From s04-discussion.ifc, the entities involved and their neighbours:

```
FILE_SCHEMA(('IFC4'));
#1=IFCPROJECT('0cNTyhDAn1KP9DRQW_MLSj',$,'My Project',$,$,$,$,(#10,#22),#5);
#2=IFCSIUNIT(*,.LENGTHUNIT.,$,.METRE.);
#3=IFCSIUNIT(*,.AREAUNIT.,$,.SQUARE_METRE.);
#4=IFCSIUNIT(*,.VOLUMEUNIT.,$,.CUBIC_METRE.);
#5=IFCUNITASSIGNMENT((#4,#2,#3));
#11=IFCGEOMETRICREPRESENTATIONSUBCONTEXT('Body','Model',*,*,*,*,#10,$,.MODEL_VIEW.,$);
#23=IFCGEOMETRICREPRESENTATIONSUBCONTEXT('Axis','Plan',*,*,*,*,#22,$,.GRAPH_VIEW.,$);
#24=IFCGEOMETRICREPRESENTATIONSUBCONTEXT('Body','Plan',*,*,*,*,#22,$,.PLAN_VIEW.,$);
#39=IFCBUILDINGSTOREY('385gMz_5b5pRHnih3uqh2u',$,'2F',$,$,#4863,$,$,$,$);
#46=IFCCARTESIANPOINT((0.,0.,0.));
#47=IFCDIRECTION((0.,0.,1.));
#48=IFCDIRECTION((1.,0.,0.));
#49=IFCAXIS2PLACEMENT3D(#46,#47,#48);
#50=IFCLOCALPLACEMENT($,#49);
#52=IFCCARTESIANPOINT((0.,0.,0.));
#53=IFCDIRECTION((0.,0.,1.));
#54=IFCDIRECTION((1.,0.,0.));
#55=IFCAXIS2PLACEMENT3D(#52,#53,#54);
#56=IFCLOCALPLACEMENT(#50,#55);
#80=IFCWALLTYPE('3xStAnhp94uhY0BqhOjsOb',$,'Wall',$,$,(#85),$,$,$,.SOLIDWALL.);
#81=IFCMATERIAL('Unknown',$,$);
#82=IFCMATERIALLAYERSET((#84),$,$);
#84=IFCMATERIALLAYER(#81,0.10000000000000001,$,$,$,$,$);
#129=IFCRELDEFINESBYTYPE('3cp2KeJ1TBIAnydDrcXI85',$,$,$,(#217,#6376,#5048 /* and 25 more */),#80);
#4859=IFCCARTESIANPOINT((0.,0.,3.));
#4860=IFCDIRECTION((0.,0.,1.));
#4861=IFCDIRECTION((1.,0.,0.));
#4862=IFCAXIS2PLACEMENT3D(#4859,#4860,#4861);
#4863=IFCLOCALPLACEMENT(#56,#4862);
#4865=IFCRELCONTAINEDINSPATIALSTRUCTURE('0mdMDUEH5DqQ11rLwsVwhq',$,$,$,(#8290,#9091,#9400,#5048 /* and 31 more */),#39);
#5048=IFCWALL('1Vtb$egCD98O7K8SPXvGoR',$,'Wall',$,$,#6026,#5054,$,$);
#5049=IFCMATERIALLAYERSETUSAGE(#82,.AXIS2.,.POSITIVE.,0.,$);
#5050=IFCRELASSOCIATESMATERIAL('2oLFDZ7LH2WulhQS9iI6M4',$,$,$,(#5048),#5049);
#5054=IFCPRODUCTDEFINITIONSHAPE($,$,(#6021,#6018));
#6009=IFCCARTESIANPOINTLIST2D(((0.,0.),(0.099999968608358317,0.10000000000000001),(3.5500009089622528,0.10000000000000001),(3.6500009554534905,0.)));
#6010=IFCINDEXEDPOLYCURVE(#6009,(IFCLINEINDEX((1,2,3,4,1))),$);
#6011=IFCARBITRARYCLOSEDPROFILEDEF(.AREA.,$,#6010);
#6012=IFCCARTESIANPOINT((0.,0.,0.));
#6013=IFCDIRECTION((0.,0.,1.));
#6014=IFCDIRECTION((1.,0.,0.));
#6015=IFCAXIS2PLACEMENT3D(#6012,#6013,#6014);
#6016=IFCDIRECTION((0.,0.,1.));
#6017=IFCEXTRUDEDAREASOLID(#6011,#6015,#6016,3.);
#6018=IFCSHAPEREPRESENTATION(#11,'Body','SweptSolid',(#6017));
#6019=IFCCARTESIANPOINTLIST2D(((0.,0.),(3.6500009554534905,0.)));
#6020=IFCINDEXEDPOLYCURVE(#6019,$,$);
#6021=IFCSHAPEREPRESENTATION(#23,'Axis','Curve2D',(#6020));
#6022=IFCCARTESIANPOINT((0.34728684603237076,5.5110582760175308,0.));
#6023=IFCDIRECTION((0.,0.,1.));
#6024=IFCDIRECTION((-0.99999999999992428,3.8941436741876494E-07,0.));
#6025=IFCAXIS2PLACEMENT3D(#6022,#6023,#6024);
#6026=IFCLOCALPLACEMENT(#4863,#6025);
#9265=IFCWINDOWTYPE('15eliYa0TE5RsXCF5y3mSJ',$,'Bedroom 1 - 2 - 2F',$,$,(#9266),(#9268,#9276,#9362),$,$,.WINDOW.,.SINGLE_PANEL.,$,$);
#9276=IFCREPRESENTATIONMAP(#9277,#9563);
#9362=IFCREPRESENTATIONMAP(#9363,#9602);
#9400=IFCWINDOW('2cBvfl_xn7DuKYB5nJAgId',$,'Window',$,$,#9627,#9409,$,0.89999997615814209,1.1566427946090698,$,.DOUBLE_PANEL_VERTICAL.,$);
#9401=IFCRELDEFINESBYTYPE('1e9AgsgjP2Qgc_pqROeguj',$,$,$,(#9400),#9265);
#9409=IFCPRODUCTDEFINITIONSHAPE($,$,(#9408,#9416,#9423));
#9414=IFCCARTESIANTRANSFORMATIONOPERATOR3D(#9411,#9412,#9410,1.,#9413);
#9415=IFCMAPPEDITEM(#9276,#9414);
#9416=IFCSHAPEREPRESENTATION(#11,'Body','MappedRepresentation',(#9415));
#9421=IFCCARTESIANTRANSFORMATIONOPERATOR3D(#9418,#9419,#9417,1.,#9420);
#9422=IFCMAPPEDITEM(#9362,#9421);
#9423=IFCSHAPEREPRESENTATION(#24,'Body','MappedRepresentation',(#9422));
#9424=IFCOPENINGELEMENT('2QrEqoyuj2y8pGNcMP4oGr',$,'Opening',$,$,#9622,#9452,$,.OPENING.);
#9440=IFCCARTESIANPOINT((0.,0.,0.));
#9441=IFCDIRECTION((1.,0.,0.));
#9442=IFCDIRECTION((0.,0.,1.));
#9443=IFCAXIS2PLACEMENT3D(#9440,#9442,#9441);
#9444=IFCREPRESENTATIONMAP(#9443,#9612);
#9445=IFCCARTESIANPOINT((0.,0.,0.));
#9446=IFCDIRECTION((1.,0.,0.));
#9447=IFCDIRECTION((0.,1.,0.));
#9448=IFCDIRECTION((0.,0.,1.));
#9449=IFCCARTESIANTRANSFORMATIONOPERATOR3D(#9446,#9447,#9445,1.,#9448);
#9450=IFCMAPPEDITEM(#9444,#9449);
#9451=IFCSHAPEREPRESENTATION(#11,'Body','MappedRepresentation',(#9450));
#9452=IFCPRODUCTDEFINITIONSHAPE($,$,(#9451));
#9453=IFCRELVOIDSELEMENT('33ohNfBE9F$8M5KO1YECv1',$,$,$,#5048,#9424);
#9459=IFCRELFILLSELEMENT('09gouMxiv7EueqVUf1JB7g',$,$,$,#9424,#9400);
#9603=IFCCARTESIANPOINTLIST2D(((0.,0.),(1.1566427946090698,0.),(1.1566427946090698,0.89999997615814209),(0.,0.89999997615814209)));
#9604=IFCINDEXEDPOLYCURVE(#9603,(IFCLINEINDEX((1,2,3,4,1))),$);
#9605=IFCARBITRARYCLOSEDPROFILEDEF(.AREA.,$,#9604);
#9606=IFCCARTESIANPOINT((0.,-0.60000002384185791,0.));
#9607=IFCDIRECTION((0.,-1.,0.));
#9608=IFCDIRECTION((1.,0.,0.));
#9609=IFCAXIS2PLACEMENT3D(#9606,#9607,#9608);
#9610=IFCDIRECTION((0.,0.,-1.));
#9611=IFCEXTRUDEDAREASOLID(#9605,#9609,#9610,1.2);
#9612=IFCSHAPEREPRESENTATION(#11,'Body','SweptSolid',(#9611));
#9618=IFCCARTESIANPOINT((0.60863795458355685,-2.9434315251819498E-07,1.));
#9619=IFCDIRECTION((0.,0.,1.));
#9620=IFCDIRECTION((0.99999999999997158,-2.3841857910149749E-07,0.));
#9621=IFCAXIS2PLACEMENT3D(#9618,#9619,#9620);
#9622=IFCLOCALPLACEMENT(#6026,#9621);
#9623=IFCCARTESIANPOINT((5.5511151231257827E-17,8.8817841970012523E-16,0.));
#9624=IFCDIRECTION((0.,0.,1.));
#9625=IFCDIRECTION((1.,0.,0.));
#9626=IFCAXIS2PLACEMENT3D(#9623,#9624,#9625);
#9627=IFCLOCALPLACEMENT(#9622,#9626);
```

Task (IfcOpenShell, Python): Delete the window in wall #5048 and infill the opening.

```python
import ifcopenshell
import ifcopenshell.api.feature
import ifcopenshell.api.root
import ifcopenshell.geom
import ifcopenshell.util.shape

model = ifcopenshell.open("s04-discussion.ifc")
settings = ifcopenshell.geom.settings()


def volume(element):
    """Net volume in cubic metres, openings subtracted."""
    shape = ifcopenshell.geom.create_shape(settings, element)
    return ifcopenshell.util.shape.get_volume(shape.geometry)


window = model.by_guid("2cBvfl_xn7DuKYB5nJAgId")
opening = window.FillsVoids[0].RelatingOpeningElement
wall = opening.VoidsElements[0].RelatingBuildingElement
before = volume(wall)

ifcopenshell.api.root.remove_product(model, product=window)
ifcopenshell.api.feature.remove_feature(model, feature=opening)

after = volume(wall)

print(f"wall volume {before:.3f} -> {after:.3f} m3")

model.write("s04-discussion_updated.ifc")
```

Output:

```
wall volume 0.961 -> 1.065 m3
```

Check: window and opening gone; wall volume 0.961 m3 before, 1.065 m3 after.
